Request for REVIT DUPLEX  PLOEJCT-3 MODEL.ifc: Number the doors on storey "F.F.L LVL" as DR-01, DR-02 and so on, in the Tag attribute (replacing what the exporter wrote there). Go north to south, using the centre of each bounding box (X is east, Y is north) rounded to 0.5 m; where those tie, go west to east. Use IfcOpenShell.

First a look at what the model holds.

```python
import ifcopenshell
import ifcopenshell.util.element
import ifcopenshell.util.placement

model = ifcopenshell.open("REVIT DUPLEX  PLOEJCT-3 MODEL.ifc")
print(model.schema)
storey = next(s for s in model.by_type("IfcBuildingStorey") if s.Name == "F.F.L LVL")
doors = [e for e in ifcopenshell.util.element.get_decomposition(storey) if e.is_a("IfcDoor")]
for e in sorted(doors, key=lambda e: e.id()):
    origin = ifcopenshell.util.placement.get_local_placement(e.ObjectPlacement)[:3, 3]
    print(e.id(), e.Tag, e.Name, origin.round(2) + 0.0, sep=" | ")
```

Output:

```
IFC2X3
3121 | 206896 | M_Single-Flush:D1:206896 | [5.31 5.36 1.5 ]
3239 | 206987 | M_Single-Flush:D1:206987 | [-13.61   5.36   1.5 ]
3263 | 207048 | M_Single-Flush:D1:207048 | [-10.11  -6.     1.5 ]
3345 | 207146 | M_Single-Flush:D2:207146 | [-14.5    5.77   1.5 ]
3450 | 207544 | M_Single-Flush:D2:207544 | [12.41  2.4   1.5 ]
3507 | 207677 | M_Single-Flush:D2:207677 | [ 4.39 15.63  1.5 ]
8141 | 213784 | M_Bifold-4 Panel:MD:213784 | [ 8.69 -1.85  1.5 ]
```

```python
import ifcopenshell
import ifcopenshell.geom
import ifcopenshell.util.element
import ifcopenshell.util.shape

model = ifcopenshell.open("REVIT DUPLEX  PLOEJCT-3 MODEL.ifc")
settings = ifcopenshell.geom.settings()
settings.set("use-world-coords", True)


def centre(element):
    shape = ifcopenshell.geom.create_shape(settings, element)
    return ifcopenshell.util.shape.get_bbox_centroid(shape.geometry)


storey = next(s for s in model.by_type("IfcBuildingStorey") if s.Name == "F.F.L LVL")
doors = [e for e in ifcopenshell.util.element.get_decomposition(storey) if e.is_a("IfcDoor")]

# Insertion points can sit at a corner or the storey origin, so sort by the geometry (in metres).
centres = {e: centre(e) for e in doors}
doors.sort(key=lambda e: (-round(centres[e][1] / 0.5), centres[e][0]))

for i, e in enumerate(doors, start=1):
    number = f"DR-{i:02d}"
    e.Tag = number
    print(e.id(), number)

model.write("REVIT DUPLEX  PLOEJCT-3 MODEL_rev.ifc")
```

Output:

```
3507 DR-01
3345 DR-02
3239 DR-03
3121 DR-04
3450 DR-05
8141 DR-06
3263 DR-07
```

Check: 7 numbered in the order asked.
